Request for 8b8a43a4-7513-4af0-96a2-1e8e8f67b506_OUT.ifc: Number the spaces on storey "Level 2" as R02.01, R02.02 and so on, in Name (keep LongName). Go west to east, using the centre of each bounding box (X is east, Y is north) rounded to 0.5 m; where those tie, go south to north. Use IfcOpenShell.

First a look at what the model holds.

```python
import ifcopenshell
import ifcopenshell.util.element
import ifcopenshell.util.placement

model = ifcopenshell.open("8b8a43a4-7513-4af0-96a2-1e8e8f67b506_OUT.ifc")
print(model.schema)
storey = next(s for s in model.by_type("IfcBuildingStorey") if s.Name == "Level 2")
spaces = [e for e in ifcopenshell.util.element.get_decomposition(storey) if e.is_a("IfcSpace")]
for e in sorted(spaces, key=lambda e: e.id()):
    origin = ifcopenshell.util.placement.get_local_placement(e.ObjectPlacement)[:3, 3]
    print(e.id(), e.Name, e.LongName, origin.round(2) + 0.0, sep=" | ")
```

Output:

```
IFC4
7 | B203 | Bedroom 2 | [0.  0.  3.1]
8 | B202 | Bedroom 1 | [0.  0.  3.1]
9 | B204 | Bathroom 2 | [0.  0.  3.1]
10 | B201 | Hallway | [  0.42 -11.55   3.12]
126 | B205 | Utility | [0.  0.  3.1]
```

```python
import ifcopenshell
import ifcopenshell.geom
import ifcopenshell.util.element
import ifcopenshell.util.shape

model = ifcopenshell.open("8b8a43a4-7513-4af0-96a2-1e8e8f67b506_OUT.ifc")
settings = ifcopenshell.geom.settings()
settings.set("use-world-coords", True)


def centre(element):
    shape = ifcopenshell.geom.create_shape(settings, element)
    return ifcopenshell.util.shape.get_bbox_centroid(shape.geometry)


storey = next(s for s in model.by_type("IfcBuildingStorey") if s.Name == "Level 2")
spaces = [e for e in ifcopenshell.util.element.get_decomposition(storey) if e.is_a("IfcSpace")]

# Insertion points can sit at a corner or the storey origin, so sort by the geometry (in metres).
centres = {e: centre(e) for e in spaces}
spaces.sort(key=lambda e: (round(centres[e][0] / 0.5), centres[e][1]))

for i, e in enumerate(spaces, start=1):
    number = f"R02.{i:02d}"
    e.Name = number
    print(e.id(), number)

model.write("8b8a43a4-7513-4af0-96a2-1e8e8f67b506_OUT-out.ifc")
```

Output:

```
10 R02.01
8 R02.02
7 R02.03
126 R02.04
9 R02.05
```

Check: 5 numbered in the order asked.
